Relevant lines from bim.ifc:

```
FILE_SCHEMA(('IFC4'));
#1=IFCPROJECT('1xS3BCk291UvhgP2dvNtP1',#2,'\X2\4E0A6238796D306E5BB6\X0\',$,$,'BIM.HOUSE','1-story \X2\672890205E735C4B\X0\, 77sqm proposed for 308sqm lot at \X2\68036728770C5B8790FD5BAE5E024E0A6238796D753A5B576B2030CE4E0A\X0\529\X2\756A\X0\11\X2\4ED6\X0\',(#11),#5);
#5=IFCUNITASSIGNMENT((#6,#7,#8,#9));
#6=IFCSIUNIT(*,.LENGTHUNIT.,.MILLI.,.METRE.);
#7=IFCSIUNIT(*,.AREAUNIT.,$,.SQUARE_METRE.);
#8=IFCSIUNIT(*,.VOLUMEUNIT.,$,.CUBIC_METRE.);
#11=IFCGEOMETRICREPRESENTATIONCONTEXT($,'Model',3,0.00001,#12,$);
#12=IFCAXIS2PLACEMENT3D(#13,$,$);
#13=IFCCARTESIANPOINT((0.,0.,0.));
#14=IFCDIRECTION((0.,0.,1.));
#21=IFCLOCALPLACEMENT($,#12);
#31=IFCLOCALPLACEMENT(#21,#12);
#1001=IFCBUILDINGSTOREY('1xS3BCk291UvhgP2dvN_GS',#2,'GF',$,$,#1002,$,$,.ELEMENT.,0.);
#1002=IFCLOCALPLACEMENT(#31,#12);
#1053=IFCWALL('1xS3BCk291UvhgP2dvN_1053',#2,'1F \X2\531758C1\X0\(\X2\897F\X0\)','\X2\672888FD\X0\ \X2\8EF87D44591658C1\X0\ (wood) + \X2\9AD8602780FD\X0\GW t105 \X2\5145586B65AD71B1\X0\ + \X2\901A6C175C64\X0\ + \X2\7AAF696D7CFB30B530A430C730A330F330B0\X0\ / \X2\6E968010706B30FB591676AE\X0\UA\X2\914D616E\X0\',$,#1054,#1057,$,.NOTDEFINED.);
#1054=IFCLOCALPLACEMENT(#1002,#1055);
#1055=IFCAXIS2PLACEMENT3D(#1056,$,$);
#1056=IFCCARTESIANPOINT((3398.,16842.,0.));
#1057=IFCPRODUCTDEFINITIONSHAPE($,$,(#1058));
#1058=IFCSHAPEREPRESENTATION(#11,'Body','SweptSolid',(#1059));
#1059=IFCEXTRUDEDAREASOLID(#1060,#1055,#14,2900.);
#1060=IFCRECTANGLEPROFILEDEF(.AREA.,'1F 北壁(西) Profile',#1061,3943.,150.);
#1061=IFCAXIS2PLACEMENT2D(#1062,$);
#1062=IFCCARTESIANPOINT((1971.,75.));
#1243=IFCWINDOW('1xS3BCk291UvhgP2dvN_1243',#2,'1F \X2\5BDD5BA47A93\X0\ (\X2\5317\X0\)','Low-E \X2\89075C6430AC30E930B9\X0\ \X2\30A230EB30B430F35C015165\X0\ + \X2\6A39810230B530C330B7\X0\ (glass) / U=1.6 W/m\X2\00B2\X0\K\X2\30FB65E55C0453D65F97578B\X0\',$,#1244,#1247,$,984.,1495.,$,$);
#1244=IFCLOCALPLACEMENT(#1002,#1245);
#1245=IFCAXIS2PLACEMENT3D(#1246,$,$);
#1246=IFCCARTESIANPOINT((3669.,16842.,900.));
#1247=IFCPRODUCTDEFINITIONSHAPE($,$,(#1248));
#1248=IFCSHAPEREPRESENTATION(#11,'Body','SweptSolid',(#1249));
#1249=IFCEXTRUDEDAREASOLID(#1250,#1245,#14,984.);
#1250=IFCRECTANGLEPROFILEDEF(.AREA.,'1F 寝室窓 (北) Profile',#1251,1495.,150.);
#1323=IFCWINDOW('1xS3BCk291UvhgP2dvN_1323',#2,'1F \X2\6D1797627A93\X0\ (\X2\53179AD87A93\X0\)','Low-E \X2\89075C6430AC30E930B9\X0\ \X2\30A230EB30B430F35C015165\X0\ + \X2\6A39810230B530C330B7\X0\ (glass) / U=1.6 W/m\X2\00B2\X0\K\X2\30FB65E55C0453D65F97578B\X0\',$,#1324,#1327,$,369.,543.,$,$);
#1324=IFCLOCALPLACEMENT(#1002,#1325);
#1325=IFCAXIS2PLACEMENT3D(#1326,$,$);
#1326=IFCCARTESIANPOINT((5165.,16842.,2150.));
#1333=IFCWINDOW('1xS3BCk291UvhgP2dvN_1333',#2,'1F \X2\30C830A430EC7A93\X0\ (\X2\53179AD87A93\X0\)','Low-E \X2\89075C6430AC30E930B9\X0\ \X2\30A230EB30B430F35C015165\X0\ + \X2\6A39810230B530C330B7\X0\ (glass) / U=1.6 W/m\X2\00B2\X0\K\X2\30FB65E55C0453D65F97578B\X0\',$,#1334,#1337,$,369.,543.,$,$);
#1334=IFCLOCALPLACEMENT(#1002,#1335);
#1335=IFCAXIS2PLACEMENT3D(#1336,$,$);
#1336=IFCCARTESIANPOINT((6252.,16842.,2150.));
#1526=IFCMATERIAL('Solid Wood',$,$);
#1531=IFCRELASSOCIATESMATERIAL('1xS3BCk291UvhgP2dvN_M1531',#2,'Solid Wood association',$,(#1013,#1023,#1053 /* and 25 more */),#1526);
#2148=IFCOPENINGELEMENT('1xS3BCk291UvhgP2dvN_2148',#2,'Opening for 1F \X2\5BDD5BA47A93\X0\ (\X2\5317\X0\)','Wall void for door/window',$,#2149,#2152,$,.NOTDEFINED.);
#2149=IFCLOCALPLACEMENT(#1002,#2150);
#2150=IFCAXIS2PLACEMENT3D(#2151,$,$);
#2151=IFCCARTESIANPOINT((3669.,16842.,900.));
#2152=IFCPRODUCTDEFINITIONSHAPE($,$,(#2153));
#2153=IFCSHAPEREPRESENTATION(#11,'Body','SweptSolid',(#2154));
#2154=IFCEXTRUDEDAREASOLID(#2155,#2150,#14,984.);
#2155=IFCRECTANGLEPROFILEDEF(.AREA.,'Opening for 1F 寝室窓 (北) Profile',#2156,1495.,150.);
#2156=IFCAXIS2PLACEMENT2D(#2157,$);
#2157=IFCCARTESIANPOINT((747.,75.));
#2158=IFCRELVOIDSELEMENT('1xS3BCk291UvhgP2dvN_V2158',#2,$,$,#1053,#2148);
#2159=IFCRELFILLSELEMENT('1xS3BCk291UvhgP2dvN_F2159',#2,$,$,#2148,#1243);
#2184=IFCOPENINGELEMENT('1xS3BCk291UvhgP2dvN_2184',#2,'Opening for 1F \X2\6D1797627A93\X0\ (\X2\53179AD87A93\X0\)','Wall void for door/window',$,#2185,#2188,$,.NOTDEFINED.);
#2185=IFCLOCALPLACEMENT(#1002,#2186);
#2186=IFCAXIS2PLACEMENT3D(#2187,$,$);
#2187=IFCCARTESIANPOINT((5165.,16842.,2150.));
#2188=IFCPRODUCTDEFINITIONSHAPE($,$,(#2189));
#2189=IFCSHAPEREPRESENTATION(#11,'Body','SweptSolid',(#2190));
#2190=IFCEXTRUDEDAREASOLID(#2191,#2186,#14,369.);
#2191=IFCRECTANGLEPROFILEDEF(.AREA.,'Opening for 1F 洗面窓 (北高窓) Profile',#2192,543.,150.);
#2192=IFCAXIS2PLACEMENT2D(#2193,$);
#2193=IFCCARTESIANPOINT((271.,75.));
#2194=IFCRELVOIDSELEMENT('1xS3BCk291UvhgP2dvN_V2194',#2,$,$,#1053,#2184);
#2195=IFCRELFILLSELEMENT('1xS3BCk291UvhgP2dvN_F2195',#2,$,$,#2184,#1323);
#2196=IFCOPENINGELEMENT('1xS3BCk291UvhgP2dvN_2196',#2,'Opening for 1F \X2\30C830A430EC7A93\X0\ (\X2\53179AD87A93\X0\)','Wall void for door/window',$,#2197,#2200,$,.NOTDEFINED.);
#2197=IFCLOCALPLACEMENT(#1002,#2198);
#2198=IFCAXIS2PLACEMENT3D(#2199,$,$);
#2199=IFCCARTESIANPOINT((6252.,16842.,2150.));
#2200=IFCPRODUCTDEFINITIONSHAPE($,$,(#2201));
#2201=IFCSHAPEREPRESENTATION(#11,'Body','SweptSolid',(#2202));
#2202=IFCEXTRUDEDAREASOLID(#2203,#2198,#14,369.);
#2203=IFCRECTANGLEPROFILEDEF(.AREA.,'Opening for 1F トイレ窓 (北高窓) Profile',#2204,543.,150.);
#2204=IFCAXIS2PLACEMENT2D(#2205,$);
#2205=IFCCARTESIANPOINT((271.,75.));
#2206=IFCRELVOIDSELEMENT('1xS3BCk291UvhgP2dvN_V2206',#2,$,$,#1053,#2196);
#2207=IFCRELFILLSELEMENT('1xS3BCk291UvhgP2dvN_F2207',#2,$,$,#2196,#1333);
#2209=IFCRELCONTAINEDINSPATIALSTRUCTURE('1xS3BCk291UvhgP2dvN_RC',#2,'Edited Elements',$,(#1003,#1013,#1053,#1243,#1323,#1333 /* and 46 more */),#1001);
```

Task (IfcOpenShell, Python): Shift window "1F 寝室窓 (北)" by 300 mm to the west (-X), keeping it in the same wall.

```python
import ifcopenshell
import ifcopenshell.api.geometry
import ifcopenshell.util.placement

model = ifcopenshell.open("bim.ifc")

window = model.by_guid("1xS3BCk291UvhgP2dvN_1243")
opening = window.FillsVoids[0].RelatingOpeningElement
wall = opening.VoidsElements[0].RelatingBuildingElement

wall_matrix = ifcopenshell.util.placement.get_local_placement(wall.ObjectPlacement)
shift = wall_matrix[:3, 0] * -300.0
before = ifcopenshell.util.placement.get_local_placement(window.ObjectPlacement)[:3, 3].copy()

# The window is not placed relative to its opening, so move both.
for product in (opening, window):
    matrix = ifcopenshell.util.placement.get_local_placement(product.ObjectPlacement)
    matrix[:3, 3] += shift
    ifcopenshell.api.geometry.edit_object_placement(model, product=product, matrix=matrix, is_si=False)

after = ifcopenshell.util.placement.get_local_placement(window.ObjectPlacement)[:3, 3]
print("window moved by", (after - before).round(3) + 0.0)

model.write("bim_updated.ifc")
```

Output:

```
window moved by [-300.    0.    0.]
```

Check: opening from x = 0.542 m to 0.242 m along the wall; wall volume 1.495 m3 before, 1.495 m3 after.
